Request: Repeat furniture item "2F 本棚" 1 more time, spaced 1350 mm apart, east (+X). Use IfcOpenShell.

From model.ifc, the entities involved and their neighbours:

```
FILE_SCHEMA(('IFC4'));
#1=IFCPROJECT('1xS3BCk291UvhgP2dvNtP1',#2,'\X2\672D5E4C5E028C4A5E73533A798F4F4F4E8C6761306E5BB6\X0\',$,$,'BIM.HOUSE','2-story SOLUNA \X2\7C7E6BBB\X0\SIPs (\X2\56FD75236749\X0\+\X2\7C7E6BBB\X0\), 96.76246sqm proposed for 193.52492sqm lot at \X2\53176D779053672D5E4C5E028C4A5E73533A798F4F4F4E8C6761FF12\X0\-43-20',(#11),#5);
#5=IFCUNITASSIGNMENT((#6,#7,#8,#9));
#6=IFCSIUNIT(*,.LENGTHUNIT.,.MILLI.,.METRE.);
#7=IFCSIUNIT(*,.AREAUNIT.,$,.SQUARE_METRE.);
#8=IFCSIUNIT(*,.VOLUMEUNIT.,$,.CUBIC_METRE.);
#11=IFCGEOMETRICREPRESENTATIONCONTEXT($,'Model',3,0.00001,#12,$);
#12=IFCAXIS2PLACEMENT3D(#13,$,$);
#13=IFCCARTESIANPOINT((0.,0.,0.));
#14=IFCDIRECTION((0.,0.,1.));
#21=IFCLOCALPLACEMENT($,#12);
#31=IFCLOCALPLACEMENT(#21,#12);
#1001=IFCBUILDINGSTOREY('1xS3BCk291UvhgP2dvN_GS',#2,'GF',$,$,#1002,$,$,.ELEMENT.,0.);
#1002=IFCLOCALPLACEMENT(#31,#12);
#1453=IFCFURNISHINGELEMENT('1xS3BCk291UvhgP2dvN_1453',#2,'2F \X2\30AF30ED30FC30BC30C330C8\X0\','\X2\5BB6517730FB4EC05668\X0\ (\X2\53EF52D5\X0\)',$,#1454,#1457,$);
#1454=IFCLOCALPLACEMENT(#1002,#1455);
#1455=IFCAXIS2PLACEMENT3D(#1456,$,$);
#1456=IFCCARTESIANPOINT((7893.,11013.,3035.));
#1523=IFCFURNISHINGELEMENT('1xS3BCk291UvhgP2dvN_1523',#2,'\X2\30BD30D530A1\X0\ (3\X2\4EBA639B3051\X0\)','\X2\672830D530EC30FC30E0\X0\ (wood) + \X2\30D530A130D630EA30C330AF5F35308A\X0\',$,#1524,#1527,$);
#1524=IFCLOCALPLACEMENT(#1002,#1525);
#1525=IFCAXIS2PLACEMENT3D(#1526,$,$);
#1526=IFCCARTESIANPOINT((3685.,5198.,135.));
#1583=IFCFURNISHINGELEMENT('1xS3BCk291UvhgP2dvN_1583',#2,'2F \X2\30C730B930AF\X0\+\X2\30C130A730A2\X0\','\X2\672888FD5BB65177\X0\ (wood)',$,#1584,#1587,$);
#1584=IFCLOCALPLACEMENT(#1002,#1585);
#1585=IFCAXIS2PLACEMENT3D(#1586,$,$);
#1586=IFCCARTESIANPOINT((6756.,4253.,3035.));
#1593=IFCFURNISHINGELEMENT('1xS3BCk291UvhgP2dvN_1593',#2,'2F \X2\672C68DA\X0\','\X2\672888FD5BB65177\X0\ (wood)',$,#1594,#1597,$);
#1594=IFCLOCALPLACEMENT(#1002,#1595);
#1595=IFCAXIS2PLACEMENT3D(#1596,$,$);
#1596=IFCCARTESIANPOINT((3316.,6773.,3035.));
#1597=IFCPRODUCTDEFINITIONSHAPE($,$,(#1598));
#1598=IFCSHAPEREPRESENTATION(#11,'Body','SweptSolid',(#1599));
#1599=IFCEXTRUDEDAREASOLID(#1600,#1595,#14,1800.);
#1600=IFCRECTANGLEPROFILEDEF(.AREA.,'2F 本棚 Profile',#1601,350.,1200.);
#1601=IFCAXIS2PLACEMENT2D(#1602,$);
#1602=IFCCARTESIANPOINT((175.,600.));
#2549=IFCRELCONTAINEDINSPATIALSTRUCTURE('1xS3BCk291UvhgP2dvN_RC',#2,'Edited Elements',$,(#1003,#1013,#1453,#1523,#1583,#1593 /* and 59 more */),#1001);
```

```python
import numpy as np
import ifcopenshell
import ifcopenshell.api.geometry
import ifcopenshell.api.root
import ifcopenshell.util.element
import ifcopenshell.util.placement
import ifcopenshell.util.unit

model = ifcopenshell.open("model.ifc")
unit_scale = ifcopenshell.util.unit.calculate_unit_scale(model)


def reuse_history(source, copy):
    """copy_class also copies each property set's owner history, people and application; keep the originals."""
    for rel in copy.IsDefinedBy:
        if rel.is_a("IfcRelDefinesByProperties") and (history := rel.RelatingPropertyDefinition.OwnerHistory):
            rel.RelatingPropertyDefinition.OwnerHistory = source.OwnerHistory
            ifcopenshell.util.element.remove_deep2(model, history)


source = model.by_guid("1xS3BCk291UvhgP2dvN_1593")
base = ifcopenshell.util.placement.get_local_placement(source.ObjectPlacement)
step = np.array([1.0, 0.0, 0.0]) * 1.35 / unit_scale

for i in range(1, 2):
    copy = ifcopenshell.api.root.copy_class(model, product=source)
    copy.Representation = ifcopenshell.util.element.copy_deep(
        model, source.Representation, exclude=["IfcGeometricRepresentationContext", "IfcRepresentationMap"]
    )
    reuse_history(source, copy)
    matrix = base.copy()
    matrix[:3, 3] += i * step
    print("added at", matrix[:3, 3].round(3) + 0.0)
    ifcopenshell.api.geometry.edit_object_placement(model, product=copy, matrix=matrix, is_si=False)

model.write("model-out.ifc")
```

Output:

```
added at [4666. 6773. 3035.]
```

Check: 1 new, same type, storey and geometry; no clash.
